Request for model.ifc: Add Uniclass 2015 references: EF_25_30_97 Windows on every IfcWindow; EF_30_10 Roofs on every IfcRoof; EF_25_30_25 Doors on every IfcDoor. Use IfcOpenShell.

First a look at what the model holds.

```python
import ifcopenshell

model = ifcopenshell.open("model.ifc")
print(model.schema)
print("classifications:", [c.Name for c in model.by_type("IfcClassification")])
for ifc_class in ("IfcDoor", "IfcRoof", "IfcStair", "IfcWall", "IfcWindow"):
    print(ifc_class, len(model.by_type(ifc_class)))
```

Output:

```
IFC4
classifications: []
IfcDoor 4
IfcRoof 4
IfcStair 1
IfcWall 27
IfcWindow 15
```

```python
import ifcopenshell
import ifcopenshell.api.classification

model = ifcopenshell.open("model.ifc")

system = ifcopenshell.api.classification.add_classification(model, classification="Uniclass 2015")

codes = {
    "IfcWindow": ("EF_25_30_97", "Windows"),
    "IfcRoof": ("EF_30_10", "Roofs"),
    "IfcDoor": ("EF_25_30_25", "Doors"),
}
for ifc_class, (code, name) in codes.items():
    products = model.by_type(ifc_class)
    ifcopenshell.api.classification.add_reference(
        model, products=products, classification=system, identification=code, name=name
    )
    print(code, len(products))

model.write("model_rev.ifc")
```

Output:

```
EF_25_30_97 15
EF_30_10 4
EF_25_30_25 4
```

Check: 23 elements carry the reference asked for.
